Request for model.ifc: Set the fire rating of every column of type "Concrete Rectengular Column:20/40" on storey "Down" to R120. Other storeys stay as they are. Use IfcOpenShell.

First a look at what the model holds.

```python
import ifcopenshell
import ifcopenshell.util.element

model = ifcopenshell.open("model.ifc")
print(model.schema)
storey = next(s for s in model.by_type("IfcBuildingStorey") if s.Name == "Down")
columns = [e for e in ifcopenshell.util.element.get_decomposition(storey) if e.is_a("IfcColumn")]
seen = {}
for e in columns:
    element_type = ifcopenshell.util.element.get_type(e)
    key = (element_type.Name if element_type != e and element_type else None, ifcopenshell.util.element.get_pset(e, "Pset_ColumnCommon", "FireRating"))
    seen[key] = seen.get(key, 0) + 1
for (name, value), count in sorted(seen.items(), key=str):
    print(count, "x", name, "|", value)
```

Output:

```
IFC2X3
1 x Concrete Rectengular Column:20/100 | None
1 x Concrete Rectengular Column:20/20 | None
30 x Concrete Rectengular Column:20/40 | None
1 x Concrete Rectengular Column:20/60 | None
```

```python
import ifcopenshell
import ifcopenshell.api.pset
import ifcopenshell.util.element

model = ifcopenshell.open("model.ifc")

storey = next(s for s in model.by_type("IfcBuildingStorey") if s.Name == "Down")
columns = [e for e in ifcopenshell.util.element.get_decomposition(storey) if e.is_a("IfcColumn")]

count = 0
for e in columns:
    element_type = ifcopenshell.util.element.get_type(e)
    if element_type in (None, e) or element_type.Name != "Concrete Rectengular Column:20/40":
        continue
    # add_pset returns the element's existing set when there is one.
    pset = ifcopenshell.api.pset.add_pset(model, product=e, name="Pset_ColumnCommon")
    ifcopenshell.api.pset.edit_pset(model, pset=pset, properties={"FireRating": "R120"})
    count += 1

print(count, "columns updated")

model.write("model_updated.ifc")
```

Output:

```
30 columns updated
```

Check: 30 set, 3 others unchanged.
